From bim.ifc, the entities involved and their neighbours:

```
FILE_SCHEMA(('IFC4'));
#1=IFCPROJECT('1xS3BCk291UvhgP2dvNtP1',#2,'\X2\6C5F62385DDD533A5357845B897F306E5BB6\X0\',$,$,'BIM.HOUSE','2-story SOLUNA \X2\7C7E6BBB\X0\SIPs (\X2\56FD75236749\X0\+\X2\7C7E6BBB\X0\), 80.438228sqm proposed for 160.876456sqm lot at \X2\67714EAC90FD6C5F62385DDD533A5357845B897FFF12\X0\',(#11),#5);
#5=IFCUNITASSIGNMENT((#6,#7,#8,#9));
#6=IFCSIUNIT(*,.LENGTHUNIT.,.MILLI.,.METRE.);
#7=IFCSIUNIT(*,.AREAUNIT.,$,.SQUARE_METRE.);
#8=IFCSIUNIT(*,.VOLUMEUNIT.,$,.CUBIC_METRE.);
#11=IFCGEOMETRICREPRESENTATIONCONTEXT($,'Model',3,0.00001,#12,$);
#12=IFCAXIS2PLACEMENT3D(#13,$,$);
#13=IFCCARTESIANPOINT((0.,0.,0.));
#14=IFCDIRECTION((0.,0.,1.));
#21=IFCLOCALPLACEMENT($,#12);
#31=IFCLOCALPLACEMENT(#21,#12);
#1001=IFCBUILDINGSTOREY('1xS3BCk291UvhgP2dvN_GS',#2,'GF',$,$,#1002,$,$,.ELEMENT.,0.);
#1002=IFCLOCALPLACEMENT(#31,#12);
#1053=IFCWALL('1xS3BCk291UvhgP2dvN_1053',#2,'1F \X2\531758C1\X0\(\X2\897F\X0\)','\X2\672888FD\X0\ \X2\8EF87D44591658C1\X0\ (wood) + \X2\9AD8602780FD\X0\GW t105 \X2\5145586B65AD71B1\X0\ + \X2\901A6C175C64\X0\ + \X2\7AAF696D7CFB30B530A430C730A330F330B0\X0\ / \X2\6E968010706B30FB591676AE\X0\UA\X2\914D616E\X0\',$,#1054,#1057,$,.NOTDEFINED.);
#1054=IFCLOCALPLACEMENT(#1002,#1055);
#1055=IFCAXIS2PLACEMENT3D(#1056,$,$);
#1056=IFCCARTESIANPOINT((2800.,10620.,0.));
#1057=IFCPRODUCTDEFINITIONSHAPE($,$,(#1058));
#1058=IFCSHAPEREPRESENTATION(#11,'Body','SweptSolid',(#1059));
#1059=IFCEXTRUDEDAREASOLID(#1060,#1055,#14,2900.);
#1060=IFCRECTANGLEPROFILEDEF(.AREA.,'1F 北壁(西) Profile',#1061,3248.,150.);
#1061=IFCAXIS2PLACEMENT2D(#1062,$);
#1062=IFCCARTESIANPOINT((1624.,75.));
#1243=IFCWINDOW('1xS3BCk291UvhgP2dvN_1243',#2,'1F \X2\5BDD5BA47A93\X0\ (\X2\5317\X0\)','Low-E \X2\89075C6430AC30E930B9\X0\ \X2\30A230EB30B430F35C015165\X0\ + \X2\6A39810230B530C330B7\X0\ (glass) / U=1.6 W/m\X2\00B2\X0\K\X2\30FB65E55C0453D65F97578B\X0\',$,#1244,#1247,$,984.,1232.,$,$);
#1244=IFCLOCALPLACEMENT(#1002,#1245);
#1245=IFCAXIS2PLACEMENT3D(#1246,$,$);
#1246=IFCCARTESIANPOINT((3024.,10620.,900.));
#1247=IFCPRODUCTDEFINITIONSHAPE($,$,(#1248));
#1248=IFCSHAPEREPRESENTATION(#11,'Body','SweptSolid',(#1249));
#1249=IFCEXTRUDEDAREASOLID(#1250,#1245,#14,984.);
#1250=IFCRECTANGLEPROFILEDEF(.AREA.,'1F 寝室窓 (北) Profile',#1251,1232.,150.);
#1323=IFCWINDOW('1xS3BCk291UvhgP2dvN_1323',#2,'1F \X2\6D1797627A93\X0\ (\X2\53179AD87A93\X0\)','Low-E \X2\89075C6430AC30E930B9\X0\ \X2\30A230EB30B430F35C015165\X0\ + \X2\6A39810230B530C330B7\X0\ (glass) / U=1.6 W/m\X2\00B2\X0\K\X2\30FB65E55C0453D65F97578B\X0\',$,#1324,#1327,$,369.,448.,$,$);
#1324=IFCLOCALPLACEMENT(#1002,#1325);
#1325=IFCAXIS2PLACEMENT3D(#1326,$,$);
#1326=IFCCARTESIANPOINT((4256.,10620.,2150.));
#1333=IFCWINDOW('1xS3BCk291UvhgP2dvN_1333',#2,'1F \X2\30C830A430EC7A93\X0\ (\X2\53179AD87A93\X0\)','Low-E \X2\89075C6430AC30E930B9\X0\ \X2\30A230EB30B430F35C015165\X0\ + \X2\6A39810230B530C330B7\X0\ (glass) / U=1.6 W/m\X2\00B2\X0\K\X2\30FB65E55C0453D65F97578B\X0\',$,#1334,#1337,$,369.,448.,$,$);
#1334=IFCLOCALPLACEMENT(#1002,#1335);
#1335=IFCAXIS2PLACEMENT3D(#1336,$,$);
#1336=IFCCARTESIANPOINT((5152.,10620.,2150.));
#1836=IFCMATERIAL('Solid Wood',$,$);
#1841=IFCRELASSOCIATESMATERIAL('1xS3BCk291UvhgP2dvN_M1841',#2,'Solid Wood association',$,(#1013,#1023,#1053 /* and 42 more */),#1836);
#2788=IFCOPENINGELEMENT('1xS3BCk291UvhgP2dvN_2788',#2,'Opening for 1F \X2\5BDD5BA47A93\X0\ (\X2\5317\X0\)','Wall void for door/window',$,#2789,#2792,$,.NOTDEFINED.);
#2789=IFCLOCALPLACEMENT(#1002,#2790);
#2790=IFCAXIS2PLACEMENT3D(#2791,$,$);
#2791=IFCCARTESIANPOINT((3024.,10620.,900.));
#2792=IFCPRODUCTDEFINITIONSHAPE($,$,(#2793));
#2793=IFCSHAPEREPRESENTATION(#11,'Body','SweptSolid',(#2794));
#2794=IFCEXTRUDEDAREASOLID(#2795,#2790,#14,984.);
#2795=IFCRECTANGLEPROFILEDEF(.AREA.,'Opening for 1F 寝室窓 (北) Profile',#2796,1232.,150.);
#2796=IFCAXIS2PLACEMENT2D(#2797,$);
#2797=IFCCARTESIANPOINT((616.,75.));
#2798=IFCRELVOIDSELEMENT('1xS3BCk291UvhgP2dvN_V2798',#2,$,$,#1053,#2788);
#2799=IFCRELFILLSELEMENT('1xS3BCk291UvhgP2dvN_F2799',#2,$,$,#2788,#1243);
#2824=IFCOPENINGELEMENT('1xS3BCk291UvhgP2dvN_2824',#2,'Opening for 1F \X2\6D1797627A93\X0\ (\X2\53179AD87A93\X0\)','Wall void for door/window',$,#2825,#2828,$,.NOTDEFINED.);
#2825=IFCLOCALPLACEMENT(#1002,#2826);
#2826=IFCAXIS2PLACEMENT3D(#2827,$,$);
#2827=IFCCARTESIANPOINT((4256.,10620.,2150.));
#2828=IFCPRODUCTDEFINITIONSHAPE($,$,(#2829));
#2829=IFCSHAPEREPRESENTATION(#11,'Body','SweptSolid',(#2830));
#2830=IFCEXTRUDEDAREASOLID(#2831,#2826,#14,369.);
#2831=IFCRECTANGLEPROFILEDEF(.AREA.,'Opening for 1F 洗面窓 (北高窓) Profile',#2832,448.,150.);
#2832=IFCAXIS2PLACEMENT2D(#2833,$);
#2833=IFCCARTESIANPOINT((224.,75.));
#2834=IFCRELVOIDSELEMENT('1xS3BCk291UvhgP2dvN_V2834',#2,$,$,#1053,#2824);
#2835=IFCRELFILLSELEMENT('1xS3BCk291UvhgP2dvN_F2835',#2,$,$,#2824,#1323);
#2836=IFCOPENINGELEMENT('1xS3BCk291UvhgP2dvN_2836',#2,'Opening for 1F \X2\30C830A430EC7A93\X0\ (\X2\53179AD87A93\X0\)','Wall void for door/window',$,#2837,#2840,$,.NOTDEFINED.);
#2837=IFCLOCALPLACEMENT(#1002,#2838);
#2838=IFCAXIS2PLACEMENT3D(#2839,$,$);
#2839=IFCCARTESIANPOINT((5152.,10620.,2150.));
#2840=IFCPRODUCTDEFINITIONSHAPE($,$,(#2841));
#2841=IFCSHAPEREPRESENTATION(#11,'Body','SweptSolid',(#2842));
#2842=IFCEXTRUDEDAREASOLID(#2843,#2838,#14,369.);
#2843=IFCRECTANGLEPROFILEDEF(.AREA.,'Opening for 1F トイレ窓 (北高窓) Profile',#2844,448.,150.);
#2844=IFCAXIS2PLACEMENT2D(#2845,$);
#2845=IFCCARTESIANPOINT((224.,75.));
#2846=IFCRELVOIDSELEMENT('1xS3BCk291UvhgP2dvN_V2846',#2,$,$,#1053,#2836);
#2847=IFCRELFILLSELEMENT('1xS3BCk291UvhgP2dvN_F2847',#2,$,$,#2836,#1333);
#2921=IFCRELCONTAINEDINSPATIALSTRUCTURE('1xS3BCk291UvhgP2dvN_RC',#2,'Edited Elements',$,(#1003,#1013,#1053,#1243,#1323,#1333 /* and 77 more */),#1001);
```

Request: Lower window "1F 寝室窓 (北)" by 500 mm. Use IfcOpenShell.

```python
import numpy as np
import ifcopenshell
import ifcopenshell.api.geometry
import ifcopenshell.util.placement
import ifcopenshell.util.unit

model = ifcopenshell.open("bim.ifc")
unit_scale = ifcopenshell.util.unit.calculate_unit_scale(model)

window = model.by_id(1243)
opening = window.FillsVoids[0].RelatingOpeningElement
dz = -0.5 / unit_scale

shift = np.array([0.0, 0.0, dz])
# The window is not placed relative to its opening, so move both.
for product in (opening, window):
    matrix = ifcopenshell.util.placement.get_local_placement(product.ObjectPlacement)
    matrix[:3, 3] += shift
    ifcopenshell.api.geometry.edit_object_placement(model, product=product, matrix=matrix, is_si=False)

print(f"moved by {dz * unit_scale:+.3f} m")

model.write("bim-out.ifc")
```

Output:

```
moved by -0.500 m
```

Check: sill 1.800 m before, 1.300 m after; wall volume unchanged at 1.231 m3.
